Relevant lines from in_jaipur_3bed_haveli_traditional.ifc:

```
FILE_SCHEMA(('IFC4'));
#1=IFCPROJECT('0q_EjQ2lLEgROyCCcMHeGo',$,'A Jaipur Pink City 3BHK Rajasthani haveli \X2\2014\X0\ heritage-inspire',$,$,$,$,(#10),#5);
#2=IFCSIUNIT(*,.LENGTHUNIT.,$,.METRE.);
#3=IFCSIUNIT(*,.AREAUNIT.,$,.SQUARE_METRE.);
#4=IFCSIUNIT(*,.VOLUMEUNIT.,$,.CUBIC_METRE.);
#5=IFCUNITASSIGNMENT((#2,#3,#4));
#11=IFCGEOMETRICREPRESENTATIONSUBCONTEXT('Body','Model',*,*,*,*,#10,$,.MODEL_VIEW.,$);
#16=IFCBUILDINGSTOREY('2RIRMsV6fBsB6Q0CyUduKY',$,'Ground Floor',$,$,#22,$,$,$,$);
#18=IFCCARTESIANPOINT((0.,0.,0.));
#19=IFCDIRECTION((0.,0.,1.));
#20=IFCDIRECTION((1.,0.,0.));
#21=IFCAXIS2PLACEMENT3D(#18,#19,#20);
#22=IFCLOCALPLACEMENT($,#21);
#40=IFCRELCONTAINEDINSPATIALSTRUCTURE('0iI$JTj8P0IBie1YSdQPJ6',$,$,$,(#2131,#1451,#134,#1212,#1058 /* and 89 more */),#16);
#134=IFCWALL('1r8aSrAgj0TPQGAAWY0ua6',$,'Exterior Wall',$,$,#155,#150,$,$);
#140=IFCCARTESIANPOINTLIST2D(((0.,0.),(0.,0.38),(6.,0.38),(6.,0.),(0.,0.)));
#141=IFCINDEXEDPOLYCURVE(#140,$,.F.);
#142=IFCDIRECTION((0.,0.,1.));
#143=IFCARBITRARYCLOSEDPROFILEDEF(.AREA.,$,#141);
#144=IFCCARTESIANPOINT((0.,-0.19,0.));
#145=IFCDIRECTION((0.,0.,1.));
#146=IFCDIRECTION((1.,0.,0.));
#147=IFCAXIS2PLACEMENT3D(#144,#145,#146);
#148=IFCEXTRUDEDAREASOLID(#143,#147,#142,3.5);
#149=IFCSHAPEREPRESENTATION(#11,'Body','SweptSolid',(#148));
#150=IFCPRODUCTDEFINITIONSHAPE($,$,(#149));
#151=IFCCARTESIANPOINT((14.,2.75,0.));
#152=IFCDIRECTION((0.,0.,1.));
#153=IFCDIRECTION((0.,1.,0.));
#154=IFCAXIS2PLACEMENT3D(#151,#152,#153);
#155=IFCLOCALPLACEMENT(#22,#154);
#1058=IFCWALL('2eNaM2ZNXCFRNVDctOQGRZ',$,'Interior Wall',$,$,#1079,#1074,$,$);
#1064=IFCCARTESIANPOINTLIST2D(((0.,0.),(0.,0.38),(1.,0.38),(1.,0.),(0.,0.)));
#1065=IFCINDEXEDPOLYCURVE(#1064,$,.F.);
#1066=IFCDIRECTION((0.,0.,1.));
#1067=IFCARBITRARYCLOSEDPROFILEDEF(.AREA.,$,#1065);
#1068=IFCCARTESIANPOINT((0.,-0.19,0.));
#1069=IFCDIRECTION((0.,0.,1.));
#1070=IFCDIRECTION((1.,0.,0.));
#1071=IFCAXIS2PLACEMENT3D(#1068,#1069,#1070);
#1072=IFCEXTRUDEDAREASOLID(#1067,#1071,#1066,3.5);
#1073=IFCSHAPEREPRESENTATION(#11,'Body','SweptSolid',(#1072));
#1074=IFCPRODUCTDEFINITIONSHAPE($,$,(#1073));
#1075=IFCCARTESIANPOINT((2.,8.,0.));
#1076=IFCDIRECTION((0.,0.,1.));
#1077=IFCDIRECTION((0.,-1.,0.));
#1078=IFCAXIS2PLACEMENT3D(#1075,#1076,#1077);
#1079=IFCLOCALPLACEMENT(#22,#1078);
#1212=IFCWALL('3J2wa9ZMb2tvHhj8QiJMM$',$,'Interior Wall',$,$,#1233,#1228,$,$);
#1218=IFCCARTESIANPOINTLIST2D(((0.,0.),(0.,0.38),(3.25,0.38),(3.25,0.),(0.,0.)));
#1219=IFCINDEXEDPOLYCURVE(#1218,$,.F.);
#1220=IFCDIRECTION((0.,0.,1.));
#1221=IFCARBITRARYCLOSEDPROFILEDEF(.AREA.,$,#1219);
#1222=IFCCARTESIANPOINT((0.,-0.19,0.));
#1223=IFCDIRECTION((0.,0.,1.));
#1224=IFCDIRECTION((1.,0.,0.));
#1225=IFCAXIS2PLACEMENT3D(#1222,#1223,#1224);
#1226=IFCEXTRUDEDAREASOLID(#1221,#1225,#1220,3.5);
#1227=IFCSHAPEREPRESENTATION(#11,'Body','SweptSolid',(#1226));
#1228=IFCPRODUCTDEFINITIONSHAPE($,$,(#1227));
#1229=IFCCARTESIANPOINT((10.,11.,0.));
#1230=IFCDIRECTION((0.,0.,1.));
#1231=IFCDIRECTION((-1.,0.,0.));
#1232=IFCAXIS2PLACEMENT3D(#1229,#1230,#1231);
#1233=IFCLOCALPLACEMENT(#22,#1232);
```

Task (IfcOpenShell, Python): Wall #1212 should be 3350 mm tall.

```python
import ifcopenshell
import ifcopenshell.geom
import ifcopenshell.util.representation
import ifcopenshell.util.shape
import ifcopenshell.util.unit

model = ifcopenshell.open("in_jaipur_3bed_haveli_traditional.ifc")
unit_scale = ifcopenshell.util.unit.calculate_unit_scale(model)
settings = ifcopenshell.geom.settings()


def volume(element):
    """Net volume in cubic metres, openings subtracted."""
    shape = ifcopenshell.geom.create_shape(settings, element)
    return ifcopenshell.util.shape.get_volume(shape.geometry)


wall = model.by_guid("3J2wa9ZMb2tvHhj8QiJMM$")
before = volume(wall)

body = ifcopenshell.util.representation.get_representation(wall, "Model", "Body")
solid = body.Items[0]
old_height = solid.Depth
solid.Depth = 3.35 / unit_scale
after = volume(wall)

print(f"height {old_height:g} -> {solid.Depth:g}, volume {before:.3f} -> {after:.3f} m3")

model.write("in_jaipur_3bed_haveli_traditional_rev.ifc")
```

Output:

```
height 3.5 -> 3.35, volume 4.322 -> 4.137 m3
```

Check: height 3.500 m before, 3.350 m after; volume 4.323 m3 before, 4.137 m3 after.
